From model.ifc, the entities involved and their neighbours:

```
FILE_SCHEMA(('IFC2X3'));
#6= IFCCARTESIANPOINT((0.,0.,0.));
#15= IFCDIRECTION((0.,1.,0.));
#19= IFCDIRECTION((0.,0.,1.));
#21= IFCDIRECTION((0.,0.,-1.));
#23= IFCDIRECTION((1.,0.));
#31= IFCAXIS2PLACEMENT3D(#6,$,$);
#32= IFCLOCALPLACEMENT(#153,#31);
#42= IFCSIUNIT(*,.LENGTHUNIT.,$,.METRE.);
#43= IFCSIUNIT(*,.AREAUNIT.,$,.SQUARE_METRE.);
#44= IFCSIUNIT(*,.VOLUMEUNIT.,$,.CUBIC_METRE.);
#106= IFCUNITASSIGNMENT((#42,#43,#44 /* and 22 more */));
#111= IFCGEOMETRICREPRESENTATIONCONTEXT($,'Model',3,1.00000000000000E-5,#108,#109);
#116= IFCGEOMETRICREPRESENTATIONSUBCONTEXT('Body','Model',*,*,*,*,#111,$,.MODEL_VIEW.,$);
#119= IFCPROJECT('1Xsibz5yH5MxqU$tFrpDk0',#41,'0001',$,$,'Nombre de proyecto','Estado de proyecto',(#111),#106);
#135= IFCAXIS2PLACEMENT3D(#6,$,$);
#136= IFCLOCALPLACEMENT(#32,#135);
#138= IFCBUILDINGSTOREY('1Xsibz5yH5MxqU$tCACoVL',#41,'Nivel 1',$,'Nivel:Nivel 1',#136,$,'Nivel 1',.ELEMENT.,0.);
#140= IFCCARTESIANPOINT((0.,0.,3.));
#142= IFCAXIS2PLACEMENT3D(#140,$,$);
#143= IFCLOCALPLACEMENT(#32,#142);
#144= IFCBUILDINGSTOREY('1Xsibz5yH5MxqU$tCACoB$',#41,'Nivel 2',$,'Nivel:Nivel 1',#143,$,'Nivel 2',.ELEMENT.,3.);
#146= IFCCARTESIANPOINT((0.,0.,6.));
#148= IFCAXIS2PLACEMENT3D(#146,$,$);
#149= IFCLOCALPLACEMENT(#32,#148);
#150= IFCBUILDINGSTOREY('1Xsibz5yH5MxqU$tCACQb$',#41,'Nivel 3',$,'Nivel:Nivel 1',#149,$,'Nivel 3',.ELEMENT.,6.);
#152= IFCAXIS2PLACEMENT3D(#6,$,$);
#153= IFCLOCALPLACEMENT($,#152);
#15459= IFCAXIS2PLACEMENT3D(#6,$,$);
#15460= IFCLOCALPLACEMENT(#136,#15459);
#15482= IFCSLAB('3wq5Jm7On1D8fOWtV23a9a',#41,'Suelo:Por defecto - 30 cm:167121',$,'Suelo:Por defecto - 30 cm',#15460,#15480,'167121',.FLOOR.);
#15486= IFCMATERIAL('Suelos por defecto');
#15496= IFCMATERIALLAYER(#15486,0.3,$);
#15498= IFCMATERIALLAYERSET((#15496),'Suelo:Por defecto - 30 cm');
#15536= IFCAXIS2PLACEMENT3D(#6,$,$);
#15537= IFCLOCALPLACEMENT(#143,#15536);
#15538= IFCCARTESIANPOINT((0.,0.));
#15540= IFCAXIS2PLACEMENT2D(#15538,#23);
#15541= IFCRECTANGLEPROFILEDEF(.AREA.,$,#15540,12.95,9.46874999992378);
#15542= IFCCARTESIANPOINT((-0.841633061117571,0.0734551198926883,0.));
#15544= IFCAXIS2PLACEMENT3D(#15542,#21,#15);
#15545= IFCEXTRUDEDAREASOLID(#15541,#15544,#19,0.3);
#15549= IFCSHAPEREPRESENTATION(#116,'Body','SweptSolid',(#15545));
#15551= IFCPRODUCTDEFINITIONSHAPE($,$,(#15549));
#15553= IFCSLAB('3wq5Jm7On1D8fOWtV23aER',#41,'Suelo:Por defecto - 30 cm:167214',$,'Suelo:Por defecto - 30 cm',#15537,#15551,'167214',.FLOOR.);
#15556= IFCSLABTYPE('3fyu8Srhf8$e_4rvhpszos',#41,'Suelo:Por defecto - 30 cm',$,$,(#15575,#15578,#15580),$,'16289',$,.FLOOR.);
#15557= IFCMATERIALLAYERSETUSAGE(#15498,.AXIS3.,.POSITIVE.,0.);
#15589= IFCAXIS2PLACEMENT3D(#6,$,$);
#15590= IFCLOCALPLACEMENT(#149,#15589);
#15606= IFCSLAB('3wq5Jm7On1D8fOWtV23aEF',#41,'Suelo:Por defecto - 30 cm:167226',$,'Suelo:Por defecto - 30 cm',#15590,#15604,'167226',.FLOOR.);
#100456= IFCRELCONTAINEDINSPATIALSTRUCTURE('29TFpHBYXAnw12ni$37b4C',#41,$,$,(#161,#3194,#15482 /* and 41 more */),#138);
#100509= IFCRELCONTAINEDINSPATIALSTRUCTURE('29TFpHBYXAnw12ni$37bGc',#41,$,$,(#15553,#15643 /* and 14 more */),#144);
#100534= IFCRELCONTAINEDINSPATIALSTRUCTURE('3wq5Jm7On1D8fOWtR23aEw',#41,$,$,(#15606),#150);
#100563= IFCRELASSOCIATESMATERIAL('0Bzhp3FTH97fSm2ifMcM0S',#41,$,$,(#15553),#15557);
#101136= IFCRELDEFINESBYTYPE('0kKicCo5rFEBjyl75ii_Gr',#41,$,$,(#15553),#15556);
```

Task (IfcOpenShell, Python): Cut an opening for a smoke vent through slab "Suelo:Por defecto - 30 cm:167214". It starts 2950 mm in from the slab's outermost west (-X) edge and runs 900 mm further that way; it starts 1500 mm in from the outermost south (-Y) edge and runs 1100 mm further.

```python
import numpy as np
import ifcopenshell
import ifcopenshell.api.feature
import ifcopenshell.api.geometry
import ifcopenshell.api.root
import ifcopenshell.geom
import ifcopenshell.util.placement
import ifcopenshell.util.representation
import ifcopenshell.util.shape
import ifcopenshell.util.unit

model = ifcopenshell.open("model.ifc")
unit_scale = ifcopenshell.util.unit.calculate_unit_scale(model)
settings = ifcopenshell.geom.settings()


def volume(element):
    """Net volume in cubic metres, openings subtracted."""
    shape = ifcopenshell.geom.create_shape(settings, element)
    return ifcopenshell.util.shape.get_volume(shape.geometry)


slab = model.by_guid("3wq5Jm7On1D8fOWtV23aER")
before = volume(slab)

# Extent in the slab's own axes, in metres. The edges named are its -X and -Y sides.
slab_shape = ifcopenshell.geom.create_shape(settings, slab)
vertices = ifcopenshell.util.shape.get_vertices(slab_shape.geometry)
x_min, y_min, bottom = vertices.min(axis=0)
top = vertices[:, 2].max()

opening = ifcopenshell.api.root.create_entity(model, ifc_class="IfcOpeningElement", name="Smoke vent opening")
context = ifcopenshell.util.representation.get_context(model, "Model", "Body", "MODEL_VIEW")
width, depth = 0.9, 1.1
outline = [(0.0, 0.0), (width, 0.0), (width, depth), (0.0, depth), (0.0, 0.0)]
# Overshoot both faces by 50 mm so the cut is clean.
shape = ifcopenshell.api.geometry.add_slab_representation(
    model, context=context, depth=top - bottom + 0.1, polyline=outline
)
ifcopenshell.api.geometry.assign_representation(model, product=opening, representation=shape)

matrix = ifcopenshell.util.placement.get_local_placement(slab.ObjectPlacement)
matrix[:, 3] = matrix @ np.append(np.array([x_min + 2.95, y_min + 1.5, bottom - 0.05]) / unit_scale, 1.0)
ifcopenshell.api.geometry.edit_object_placement(model, product=opening, matrix=matrix, is_si=False)
ifcopenshell.api.feature.add_feature(model, feature=opening, element=slab)

after = volume(slab)

print(f"slab volume {before:.3f} -> {after:.3f} m3")

model.write("model_v2.ifc")
```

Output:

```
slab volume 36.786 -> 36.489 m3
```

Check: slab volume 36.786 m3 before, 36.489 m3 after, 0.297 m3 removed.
